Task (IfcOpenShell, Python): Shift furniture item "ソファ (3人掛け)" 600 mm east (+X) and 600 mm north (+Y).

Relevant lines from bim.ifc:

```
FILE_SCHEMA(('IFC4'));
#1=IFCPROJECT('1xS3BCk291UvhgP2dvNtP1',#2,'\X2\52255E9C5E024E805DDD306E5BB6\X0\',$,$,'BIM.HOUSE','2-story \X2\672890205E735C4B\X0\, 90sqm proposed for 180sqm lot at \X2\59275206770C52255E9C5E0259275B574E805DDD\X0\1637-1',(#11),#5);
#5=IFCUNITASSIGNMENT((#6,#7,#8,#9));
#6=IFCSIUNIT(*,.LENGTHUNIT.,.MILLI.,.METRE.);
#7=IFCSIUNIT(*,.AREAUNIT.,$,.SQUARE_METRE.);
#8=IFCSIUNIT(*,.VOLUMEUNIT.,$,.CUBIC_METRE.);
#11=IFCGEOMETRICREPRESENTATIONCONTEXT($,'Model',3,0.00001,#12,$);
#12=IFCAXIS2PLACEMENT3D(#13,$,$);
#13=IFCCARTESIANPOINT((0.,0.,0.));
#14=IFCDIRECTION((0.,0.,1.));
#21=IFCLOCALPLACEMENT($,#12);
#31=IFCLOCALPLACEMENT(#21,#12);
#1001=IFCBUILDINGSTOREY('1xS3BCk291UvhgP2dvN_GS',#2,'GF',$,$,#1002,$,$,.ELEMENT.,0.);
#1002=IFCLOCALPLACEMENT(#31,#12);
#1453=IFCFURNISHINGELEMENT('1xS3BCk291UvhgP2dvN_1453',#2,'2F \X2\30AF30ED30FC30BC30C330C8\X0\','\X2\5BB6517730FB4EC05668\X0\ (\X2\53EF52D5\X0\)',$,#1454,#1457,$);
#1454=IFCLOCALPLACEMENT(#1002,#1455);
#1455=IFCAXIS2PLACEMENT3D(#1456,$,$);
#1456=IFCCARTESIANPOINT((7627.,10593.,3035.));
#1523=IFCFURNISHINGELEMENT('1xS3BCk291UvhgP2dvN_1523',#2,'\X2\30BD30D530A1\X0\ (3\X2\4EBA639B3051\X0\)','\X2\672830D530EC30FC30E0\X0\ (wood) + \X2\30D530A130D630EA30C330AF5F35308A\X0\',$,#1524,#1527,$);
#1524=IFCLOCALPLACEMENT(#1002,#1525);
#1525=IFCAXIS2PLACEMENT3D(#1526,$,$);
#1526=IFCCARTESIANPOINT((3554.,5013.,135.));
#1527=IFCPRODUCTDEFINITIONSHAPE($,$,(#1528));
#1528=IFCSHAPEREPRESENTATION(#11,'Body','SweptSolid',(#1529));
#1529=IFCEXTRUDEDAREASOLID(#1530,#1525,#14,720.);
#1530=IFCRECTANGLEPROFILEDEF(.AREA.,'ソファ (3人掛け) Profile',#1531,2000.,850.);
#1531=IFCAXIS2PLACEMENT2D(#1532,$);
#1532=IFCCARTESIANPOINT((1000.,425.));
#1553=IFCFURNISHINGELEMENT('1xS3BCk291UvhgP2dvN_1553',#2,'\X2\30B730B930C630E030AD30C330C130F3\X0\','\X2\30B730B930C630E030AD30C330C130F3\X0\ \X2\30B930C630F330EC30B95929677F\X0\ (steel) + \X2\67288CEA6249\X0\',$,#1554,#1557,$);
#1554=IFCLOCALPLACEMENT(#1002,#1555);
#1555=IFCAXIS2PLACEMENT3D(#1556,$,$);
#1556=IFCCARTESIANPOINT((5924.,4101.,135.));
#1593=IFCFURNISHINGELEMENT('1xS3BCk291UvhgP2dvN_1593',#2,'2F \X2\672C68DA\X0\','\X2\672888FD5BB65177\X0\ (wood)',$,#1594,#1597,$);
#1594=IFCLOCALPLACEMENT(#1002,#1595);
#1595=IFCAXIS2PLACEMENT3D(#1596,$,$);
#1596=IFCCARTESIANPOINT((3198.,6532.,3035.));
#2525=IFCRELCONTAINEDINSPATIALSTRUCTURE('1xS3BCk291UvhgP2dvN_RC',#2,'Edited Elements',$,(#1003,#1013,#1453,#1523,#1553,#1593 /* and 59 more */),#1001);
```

```python
import ifcopenshell
import ifcopenshell.api.geometry
import ifcopenshell.util.placement

model = ifcopenshell.open("bim.ifc")

item = model.by_id(1523)
matrix = ifcopenshell.util.placement.get_local_placement(item.ObjectPlacement)
matrix[0, 3] += 600.0
matrix[1, 3] += 600.0
ifcopenshell.api.geometry.edit_object_placement(model, product=item, matrix=matrix, is_si=False)

print(ifcopenshell.util.placement.get_local_placement(item.ObjectPlacement).round(3) + 0.0)

model.write("bim-out.ifc")
```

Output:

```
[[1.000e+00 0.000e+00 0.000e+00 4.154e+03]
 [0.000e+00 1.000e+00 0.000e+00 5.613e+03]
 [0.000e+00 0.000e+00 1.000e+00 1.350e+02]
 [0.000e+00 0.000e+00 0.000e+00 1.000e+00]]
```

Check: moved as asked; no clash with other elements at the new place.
